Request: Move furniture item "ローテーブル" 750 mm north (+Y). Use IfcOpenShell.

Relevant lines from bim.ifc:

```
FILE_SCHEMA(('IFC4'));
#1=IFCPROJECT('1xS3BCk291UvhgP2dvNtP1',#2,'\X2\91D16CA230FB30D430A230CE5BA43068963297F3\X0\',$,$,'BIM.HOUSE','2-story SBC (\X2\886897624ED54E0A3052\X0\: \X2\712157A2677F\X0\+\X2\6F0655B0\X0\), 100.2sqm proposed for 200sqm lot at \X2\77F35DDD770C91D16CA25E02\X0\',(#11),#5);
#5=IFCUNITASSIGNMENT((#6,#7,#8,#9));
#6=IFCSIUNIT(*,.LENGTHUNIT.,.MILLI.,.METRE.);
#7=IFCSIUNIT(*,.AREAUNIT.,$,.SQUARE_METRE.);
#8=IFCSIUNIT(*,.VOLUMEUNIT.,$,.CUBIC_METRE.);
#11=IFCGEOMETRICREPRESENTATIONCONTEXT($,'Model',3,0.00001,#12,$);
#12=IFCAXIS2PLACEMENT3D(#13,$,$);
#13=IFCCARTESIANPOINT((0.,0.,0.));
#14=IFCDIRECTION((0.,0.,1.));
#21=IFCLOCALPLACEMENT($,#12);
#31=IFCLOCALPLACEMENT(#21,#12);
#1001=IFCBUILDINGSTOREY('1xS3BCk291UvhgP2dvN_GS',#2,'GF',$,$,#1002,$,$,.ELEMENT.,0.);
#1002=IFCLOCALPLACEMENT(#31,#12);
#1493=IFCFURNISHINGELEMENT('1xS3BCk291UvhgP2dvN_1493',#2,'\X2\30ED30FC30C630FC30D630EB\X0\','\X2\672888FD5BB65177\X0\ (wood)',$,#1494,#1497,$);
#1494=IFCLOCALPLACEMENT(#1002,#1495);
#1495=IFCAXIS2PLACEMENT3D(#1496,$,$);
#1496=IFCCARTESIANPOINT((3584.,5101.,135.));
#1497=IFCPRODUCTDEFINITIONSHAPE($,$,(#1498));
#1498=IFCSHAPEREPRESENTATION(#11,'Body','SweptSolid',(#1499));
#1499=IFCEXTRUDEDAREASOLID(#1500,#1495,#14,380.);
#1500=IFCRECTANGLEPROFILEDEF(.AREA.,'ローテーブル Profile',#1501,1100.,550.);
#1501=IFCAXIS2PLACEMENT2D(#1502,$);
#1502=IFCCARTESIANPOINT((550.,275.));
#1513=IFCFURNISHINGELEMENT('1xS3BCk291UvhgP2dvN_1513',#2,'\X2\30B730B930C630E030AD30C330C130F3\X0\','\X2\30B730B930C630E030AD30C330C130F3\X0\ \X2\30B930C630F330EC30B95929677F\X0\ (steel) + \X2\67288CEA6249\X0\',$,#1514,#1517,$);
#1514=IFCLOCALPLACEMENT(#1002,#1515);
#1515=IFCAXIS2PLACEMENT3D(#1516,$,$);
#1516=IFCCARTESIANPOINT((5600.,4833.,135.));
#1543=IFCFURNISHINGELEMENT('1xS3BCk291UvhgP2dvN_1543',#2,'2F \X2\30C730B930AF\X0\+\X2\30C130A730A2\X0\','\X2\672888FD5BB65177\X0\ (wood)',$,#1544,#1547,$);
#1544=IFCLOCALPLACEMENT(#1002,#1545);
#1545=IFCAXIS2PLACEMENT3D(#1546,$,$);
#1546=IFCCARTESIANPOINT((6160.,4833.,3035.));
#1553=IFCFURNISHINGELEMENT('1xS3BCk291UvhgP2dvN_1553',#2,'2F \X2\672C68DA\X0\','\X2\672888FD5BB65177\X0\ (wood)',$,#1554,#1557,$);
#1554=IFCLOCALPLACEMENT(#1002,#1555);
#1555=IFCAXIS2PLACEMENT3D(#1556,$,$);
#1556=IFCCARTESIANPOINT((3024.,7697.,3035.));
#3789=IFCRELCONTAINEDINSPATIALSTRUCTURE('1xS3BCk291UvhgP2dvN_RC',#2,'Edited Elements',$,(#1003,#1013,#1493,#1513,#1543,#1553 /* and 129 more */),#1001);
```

```python
import ifcopenshell
import ifcopenshell.api.geometry
import ifcopenshell.util.placement

model = ifcopenshell.open("bim.ifc")

item = model.by_guid("1xS3BCk291UvhgP2dvN_1493")
matrix = ifcopenshell.util.placement.get_local_placement(item.ObjectPlacement)
matrix[1, 3] += 750.0
ifcopenshell.api.geometry.edit_object_placement(model, product=item, matrix=matrix, is_si=False)

print(ifcopenshell.util.placement.get_local_placement(item.ObjectPlacement).round(3) + 0.0)

model.write("bim_v2.ifc")
```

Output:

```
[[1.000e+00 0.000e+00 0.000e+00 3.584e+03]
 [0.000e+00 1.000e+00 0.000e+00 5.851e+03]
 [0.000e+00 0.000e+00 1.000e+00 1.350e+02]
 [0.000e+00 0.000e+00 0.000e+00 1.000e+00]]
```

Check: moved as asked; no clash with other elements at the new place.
